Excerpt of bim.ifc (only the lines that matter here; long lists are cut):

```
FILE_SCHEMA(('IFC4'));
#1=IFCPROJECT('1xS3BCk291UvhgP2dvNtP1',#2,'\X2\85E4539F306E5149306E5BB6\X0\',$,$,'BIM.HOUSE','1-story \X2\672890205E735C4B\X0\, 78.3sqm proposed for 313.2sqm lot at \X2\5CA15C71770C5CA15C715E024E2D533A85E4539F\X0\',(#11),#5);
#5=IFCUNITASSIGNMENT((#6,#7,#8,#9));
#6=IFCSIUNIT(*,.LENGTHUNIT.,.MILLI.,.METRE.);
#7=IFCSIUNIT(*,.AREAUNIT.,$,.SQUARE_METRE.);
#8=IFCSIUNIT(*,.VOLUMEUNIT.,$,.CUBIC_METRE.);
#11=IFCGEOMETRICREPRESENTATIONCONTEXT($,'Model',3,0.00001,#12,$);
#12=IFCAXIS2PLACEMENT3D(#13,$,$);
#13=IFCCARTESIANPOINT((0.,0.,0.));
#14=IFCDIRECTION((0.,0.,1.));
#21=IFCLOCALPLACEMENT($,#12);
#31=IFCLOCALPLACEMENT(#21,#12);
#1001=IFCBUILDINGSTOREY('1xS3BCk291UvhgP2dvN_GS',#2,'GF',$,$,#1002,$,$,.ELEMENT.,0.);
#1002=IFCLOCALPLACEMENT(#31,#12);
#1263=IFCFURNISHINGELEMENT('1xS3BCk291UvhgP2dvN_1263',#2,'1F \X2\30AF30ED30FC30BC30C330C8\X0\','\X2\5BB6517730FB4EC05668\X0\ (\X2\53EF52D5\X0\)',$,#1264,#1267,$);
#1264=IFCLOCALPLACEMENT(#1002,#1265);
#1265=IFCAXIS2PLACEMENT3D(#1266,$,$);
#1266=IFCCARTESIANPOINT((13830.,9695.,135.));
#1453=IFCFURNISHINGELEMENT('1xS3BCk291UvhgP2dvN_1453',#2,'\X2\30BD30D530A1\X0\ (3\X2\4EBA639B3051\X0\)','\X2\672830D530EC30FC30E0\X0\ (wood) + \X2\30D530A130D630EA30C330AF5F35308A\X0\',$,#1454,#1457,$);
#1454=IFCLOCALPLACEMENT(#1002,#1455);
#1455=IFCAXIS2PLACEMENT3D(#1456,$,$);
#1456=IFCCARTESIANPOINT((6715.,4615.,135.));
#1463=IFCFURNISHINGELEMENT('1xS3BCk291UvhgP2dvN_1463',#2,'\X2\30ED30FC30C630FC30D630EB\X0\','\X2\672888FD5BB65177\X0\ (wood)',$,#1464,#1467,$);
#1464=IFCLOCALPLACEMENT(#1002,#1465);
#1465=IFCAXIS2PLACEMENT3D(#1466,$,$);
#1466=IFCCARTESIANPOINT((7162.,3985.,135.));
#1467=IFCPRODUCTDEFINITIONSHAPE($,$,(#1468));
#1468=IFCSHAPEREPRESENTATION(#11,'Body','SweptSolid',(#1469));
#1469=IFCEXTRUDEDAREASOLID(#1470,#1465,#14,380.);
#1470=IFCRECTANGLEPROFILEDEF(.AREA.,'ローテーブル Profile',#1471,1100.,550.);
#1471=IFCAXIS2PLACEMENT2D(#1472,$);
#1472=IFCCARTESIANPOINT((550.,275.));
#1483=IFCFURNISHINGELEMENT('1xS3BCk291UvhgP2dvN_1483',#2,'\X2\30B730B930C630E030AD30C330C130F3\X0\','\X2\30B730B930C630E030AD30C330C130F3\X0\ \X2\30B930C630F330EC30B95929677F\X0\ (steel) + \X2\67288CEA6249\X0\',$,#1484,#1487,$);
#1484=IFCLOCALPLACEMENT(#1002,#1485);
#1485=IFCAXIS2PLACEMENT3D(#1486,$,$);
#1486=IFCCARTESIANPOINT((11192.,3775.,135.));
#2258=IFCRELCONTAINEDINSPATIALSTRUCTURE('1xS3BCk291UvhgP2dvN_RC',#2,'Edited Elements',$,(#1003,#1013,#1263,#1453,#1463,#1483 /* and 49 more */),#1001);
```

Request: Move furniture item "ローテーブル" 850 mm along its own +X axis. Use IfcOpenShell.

```python
import ifcopenshell
import ifcopenshell.api.geometry
import ifcopenshell.util.placement
import ifcopenshell.util.unit

model = ifcopenshell.open("bim.ifc")
unit_scale = ifcopenshell.util.unit.calculate_unit_scale(model)

item = model.by_id(1463)
matrix = ifcopenshell.util.placement.get_local_placement(item.ObjectPlacement)
matrix[:3, 3] += matrix[:3, 0] * 0.85 / unit_scale
ifcopenshell.api.geometry.edit_object_placement(model, product=item, matrix=matrix, is_si=False)

print(ifcopenshell.util.placement.get_local_placement(item.ObjectPlacement).round(3) + 0.0)

model.write("bim-out.ifc")
```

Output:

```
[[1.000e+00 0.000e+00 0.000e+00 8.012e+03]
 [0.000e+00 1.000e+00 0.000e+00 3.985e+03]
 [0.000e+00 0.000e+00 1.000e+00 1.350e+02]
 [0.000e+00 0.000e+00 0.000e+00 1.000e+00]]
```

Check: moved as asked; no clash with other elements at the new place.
